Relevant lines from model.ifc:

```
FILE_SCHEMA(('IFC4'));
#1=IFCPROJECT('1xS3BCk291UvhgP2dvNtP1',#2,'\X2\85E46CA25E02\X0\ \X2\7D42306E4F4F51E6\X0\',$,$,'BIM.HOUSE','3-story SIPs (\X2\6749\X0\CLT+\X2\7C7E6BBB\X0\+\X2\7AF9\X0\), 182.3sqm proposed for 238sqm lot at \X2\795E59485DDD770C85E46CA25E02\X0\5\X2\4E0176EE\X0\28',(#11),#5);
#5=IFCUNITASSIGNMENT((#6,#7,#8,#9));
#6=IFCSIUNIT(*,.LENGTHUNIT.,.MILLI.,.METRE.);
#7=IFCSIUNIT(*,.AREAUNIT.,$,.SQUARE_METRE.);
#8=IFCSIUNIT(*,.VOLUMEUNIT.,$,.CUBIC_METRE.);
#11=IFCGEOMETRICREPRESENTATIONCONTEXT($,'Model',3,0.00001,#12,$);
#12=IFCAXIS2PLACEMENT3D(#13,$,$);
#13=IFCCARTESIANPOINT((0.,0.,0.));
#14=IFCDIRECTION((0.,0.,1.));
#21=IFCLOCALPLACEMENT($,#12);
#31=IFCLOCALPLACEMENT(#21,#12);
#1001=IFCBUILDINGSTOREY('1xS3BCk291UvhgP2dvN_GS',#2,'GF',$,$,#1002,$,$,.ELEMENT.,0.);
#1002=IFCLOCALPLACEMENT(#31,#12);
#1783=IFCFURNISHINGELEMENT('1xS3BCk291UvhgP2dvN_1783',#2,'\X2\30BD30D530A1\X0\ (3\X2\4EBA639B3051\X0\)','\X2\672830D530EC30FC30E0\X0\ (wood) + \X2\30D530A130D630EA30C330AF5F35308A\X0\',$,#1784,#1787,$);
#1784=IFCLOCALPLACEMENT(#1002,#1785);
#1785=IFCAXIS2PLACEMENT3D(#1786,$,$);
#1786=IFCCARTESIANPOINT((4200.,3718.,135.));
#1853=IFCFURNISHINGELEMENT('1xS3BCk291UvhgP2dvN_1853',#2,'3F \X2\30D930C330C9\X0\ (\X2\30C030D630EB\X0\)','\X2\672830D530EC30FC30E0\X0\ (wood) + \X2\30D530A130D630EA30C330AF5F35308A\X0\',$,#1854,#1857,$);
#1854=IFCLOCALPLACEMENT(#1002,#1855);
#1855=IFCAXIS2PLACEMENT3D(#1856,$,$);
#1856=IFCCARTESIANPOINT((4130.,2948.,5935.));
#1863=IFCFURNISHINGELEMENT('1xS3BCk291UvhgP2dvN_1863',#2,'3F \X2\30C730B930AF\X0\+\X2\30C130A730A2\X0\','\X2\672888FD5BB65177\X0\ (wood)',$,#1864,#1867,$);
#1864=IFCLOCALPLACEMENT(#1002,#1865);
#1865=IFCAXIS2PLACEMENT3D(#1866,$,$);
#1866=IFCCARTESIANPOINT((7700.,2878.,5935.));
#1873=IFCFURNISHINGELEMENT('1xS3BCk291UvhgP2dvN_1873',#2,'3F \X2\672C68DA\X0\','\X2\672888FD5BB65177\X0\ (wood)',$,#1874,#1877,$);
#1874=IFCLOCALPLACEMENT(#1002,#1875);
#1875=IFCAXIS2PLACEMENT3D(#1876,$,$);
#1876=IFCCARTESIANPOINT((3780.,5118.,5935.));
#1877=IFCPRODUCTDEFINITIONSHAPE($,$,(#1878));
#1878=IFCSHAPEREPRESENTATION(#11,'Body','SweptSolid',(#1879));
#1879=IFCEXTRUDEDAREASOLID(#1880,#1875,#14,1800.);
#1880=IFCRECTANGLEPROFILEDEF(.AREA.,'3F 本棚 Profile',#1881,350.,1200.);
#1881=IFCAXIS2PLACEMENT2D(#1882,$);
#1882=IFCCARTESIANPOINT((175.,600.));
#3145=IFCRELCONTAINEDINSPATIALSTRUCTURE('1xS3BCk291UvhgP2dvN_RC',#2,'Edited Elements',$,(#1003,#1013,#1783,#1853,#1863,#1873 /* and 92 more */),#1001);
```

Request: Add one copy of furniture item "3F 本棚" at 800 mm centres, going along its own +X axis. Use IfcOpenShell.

```python
import ifcopenshell
import ifcopenshell.api.geometry
import ifcopenshell.api.root
import ifcopenshell.util.element
import ifcopenshell.util.placement

model = ifcopenshell.open("model.ifc")


def reuse_history(source, copy):
    """copy_class also copies each property set's owner history, people and application; keep the originals."""
    for rel in copy.IsDefinedBy:
        if rel.is_a("IfcRelDefinesByProperties") and (history := rel.RelatingPropertyDefinition.OwnerHistory):
            rel.RelatingPropertyDefinition.OwnerHistory = source.OwnerHistory
            ifcopenshell.util.element.remove_deep2(model, history)


source = model.by_guid("1xS3BCk291UvhgP2dvN_1873")
base = ifcopenshell.util.placement.get_local_placement(source.ObjectPlacement)
step = base[:3, 0] * 800.0

for i in range(1, 2):
    copy = ifcopenshell.api.root.copy_class(model, product=source)
    copy.Representation = ifcopenshell.util.element.copy_deep(
        model, source.Representation, exclude=["IfcGeometricRepresentationContext", "IfcRepresentationMap"]
    )
    reuse_history(source, copy)
    matrix = base.copy()
    matrix[:3, 3] += i * step
    print("added at", matrix[:3, 3].round(3) + 0.0)
    ifcopenshell.api.geometry.edit_object_placement(model, product=copy, matrix=matrix, is_si=False)

model.write("model_rev.ifc")
```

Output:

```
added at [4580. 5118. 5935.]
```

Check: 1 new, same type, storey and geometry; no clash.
